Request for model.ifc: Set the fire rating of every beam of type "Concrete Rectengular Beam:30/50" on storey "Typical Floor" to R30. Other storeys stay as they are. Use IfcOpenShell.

First a look at what the model holds.

```python
import ifcopenshell
import ifcopenshell.util.element

model = ifcopenshell.open("model.ifc")
print(model.schema)
storey = next(s for s in model.by_type("IfcBuildingStorey") if s.Name == "Typical Floor")
beams = [e for e in ifcopenshell.util.element.get_decomposition(storey) if e.is_a("IfcBeam")]
seen = {}
for e in beams:
    element_type = ifcopenshell.util.element.get_type(e)
    key = (element_type.Name if element_type != e and element_type else None, ifcopenshell.util.element.get_pset(e, "Pset_BeamCommon", "FireRating"))
    seen[key] = seen.get(key, 0) + 1
for (name, value), count in sorted(seen.items(), key=str):
    print(count, "x", name, "|", value)
```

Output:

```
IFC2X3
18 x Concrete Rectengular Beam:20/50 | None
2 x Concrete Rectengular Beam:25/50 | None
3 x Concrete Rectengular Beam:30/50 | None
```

```python
import ifcopenshell
import ifcopenshell.api.pset
import ifcopenshell.util.element

model = ifcopenshell.open("model.ifc")

storey = next(s for s in model.by_type("IfcBuildingStorey") if s.Name == "Typical Floor")
beams = [e for e in ifcopenshell.util.element.get_decomposition(storey) if e.is_a("IfcBeam")]

count = 0
for e in beams:
    element_type = ifcopenshell.util.element.get_type(e)
    if element_type in (None, e) or element_type.Name != "Concrete Rectengular Beam:30/50":
        continue
    # add_pset returns the element's existing set when there is one.
    pset = ifcopenshell.api.pset.add_pset(model, product=e, name="Pset_BeamCommon")
    ifcopenshell.api.pset.edit_pset(model, pset=pset, properties={"FireRating": "R30"})
    count += 1

print(count, "beams updated")

model.write("model_edited.ifc")
```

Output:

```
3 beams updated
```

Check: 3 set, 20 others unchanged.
